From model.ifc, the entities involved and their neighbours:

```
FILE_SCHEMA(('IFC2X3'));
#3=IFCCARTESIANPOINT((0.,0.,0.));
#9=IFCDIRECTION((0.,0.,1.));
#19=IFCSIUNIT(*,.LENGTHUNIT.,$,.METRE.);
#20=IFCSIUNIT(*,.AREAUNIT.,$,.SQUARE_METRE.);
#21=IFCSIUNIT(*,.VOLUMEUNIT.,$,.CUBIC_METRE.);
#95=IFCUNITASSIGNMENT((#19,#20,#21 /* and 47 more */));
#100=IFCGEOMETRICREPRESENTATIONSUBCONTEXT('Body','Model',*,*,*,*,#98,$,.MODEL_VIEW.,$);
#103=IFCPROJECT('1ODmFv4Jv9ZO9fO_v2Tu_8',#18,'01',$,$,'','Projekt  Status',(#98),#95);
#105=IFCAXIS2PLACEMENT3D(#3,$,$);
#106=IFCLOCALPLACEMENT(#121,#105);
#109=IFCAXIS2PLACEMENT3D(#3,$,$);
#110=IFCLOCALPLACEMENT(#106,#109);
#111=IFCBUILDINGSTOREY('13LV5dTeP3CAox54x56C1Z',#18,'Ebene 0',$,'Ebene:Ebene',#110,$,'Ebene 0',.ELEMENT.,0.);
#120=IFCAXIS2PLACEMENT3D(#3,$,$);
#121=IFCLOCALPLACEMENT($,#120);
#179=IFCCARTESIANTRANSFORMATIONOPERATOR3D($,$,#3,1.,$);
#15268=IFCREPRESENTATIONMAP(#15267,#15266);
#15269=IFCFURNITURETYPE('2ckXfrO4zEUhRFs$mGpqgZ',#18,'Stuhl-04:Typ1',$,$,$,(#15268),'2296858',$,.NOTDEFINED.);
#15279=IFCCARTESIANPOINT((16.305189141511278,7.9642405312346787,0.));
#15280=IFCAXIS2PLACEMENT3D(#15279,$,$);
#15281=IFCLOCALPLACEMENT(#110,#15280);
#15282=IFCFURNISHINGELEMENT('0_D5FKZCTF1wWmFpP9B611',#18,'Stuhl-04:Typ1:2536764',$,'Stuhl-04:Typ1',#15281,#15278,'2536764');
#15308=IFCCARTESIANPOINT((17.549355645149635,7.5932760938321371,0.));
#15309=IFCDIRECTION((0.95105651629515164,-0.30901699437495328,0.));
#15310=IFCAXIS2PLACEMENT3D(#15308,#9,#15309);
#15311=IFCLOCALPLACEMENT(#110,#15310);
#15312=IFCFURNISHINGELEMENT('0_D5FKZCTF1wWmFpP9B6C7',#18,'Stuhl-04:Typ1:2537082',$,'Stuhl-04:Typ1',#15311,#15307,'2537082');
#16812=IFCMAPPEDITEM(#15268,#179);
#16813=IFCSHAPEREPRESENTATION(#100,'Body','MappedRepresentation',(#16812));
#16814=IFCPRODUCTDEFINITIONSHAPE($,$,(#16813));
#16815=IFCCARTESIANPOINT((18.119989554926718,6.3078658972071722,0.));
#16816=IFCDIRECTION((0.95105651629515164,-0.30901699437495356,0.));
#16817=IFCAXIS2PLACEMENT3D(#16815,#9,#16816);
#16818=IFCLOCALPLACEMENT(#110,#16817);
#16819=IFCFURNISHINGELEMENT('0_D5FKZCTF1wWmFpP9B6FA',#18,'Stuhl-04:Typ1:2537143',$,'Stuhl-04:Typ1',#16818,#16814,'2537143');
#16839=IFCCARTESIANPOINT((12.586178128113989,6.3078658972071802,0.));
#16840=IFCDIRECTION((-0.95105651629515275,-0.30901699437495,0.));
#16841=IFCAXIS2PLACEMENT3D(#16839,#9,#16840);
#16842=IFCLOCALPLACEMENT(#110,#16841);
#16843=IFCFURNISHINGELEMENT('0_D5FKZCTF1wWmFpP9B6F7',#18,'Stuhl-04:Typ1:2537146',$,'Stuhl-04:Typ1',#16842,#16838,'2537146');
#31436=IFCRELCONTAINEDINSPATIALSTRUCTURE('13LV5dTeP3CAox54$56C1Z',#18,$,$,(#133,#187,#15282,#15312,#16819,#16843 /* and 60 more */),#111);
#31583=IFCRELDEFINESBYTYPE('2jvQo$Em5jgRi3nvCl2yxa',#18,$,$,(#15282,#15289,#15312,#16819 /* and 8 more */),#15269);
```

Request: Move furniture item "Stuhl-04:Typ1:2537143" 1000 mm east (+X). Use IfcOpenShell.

```python
import ifcopenshell
import ifcopenshell.api.geometry
import ifcopenshell.util.placement
import ifcopenshell.util.unit

model = ifcopenshell.open("model.ifc")
unit_scale = ifcopenshell.util.unit.calculate_unit_scale(model)

item = model.by_id(16819)
matrix = ifcopenshell.util.placement.get_local_placement(item.ObjectPlacement)
matrix[0, 3] += 1 / unit_scale
ifcopenshell.api.geometry.edit_object_placement(model, product=item, matrix=matrix, is_si=False)

print(ifcopenshell.util.placement.get_local_placement(item.ObjectPlacement).round(3) + 0.0)

model.write("model_updated.ifc")
```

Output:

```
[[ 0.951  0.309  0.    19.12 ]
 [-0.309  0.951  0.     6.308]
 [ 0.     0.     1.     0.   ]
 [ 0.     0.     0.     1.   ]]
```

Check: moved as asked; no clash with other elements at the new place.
